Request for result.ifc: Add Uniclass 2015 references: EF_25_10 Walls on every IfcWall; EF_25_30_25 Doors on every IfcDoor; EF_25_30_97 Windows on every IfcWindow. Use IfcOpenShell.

First a look at what the model holds.

```python
import ifcopenshell

model = ifcopenshell.open("result.ifc")
print(model.schema)
print("classifications:", [c.Name for c in model.by_type("IfcClassification")])
for ifc_class in ("IfcDoor", "IfcRoof", "IfcStair", "IfcWall", "IfcWindow"):
    print(ifc_class, len(model.by_type(ifc_class)))
```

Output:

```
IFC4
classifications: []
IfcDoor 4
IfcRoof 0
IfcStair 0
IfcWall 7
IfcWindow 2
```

```python
import ifcopenshell
import ifcopenshell.api.classification

model = ifcopenshell.open("result.ifc")

system = ifcopenshell.api.classification.add_classification(model, classification="Uniclass 2015")

codes = {
    "IfcWall": ("EF_25_10", "Walls"),
    "IfcDoor": ("EF_25_30_25", "Doors"),
    "IfcWindow": ("EF_25_30_97", "Windows"),
}
for ifc_class, (code, name) in codes.items():
    products = model.by_type(ifc_class)
    ifcopenshell.api.classification.add_reference(
        model, products=products, classification=system, identification=code, name=name
    )
    print(code, len(products))

model.write("result_rev.ifc")
```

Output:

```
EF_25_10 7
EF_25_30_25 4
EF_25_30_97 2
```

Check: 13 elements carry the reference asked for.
